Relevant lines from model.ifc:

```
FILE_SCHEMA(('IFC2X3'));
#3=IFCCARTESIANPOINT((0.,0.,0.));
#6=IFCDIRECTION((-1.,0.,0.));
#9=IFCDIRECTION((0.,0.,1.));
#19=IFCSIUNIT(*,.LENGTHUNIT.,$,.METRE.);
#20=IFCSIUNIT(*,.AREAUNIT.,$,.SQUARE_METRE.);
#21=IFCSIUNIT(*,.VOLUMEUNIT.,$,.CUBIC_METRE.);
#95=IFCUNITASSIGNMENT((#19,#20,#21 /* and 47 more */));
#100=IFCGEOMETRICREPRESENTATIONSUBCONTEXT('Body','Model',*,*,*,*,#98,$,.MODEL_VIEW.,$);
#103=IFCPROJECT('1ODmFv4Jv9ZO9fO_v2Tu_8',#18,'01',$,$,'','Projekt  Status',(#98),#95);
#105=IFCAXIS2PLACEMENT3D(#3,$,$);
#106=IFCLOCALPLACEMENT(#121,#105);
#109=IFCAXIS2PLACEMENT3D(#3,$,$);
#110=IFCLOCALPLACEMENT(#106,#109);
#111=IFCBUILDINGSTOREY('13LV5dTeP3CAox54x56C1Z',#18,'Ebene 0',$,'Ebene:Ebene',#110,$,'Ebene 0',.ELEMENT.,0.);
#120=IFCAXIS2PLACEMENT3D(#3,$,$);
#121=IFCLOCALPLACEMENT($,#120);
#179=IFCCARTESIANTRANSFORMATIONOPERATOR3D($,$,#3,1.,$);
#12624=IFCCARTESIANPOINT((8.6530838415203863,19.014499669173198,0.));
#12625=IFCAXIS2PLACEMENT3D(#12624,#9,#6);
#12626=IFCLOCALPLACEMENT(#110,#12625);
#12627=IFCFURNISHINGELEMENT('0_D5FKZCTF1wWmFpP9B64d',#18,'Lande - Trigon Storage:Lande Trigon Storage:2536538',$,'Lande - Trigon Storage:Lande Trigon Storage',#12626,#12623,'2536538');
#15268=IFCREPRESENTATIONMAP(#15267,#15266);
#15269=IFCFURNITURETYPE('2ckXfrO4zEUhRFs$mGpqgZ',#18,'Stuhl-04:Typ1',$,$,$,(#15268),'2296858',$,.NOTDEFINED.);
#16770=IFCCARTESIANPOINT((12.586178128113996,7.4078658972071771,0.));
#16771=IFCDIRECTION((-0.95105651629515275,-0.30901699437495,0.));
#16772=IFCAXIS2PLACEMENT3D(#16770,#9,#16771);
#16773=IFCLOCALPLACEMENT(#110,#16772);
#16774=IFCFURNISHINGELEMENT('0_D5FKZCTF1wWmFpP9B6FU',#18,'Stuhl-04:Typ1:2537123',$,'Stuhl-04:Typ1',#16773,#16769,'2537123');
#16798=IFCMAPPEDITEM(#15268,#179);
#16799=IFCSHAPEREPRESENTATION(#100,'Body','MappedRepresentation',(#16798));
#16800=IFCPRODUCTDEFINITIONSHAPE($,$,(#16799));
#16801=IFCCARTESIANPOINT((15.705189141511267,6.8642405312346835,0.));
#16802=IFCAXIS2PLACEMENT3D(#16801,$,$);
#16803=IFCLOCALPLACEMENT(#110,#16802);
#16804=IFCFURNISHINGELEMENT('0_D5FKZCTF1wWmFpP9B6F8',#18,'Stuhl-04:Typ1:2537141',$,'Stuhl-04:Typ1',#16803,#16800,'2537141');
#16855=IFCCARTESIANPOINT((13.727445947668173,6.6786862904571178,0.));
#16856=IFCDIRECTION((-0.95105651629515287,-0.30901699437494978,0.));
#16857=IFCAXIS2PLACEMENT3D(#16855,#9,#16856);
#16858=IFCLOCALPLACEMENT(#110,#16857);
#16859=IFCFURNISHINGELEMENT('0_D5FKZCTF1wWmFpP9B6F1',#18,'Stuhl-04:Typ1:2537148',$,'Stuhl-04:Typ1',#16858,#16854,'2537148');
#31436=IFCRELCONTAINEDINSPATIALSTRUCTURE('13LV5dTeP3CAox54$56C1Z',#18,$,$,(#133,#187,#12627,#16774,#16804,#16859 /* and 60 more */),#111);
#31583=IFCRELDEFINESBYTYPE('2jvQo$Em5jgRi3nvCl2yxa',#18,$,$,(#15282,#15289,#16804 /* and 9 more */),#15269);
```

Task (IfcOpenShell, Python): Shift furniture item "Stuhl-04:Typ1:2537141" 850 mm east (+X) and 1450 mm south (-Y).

```python
import ifcopenshell
import ifcopenshell.api.geometry
import ifcopenshell.util.placement
import ifcopenshell.util.unit

model = ifcopenshell.open("model.ifc")
unit_scale = ifcopenshell.util.unit.calculate_unit_scale(model)

item = model.by_guid("0_D5FKZCTF1wWmFpP9B6F8")
matrix = ifcopenshell.util.placement.get_local_placement(item.ObjectPlacement)
matrix[0, 3] += 0.85 / unit_scale
matrix[1, 3] -= 1.45 / unit_scale
ifcopenshell.api.geometry.edit_object_placement(model, product=item, matrix=matrix, is_si=False)

print(ifcopenshell.util.placement.get_local_placement(item.ObjectPlacement).round(3) + 0.0)

model.write("model-out.ifc")
```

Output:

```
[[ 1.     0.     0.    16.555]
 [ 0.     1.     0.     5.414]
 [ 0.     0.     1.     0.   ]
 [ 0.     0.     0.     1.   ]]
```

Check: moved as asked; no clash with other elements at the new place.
